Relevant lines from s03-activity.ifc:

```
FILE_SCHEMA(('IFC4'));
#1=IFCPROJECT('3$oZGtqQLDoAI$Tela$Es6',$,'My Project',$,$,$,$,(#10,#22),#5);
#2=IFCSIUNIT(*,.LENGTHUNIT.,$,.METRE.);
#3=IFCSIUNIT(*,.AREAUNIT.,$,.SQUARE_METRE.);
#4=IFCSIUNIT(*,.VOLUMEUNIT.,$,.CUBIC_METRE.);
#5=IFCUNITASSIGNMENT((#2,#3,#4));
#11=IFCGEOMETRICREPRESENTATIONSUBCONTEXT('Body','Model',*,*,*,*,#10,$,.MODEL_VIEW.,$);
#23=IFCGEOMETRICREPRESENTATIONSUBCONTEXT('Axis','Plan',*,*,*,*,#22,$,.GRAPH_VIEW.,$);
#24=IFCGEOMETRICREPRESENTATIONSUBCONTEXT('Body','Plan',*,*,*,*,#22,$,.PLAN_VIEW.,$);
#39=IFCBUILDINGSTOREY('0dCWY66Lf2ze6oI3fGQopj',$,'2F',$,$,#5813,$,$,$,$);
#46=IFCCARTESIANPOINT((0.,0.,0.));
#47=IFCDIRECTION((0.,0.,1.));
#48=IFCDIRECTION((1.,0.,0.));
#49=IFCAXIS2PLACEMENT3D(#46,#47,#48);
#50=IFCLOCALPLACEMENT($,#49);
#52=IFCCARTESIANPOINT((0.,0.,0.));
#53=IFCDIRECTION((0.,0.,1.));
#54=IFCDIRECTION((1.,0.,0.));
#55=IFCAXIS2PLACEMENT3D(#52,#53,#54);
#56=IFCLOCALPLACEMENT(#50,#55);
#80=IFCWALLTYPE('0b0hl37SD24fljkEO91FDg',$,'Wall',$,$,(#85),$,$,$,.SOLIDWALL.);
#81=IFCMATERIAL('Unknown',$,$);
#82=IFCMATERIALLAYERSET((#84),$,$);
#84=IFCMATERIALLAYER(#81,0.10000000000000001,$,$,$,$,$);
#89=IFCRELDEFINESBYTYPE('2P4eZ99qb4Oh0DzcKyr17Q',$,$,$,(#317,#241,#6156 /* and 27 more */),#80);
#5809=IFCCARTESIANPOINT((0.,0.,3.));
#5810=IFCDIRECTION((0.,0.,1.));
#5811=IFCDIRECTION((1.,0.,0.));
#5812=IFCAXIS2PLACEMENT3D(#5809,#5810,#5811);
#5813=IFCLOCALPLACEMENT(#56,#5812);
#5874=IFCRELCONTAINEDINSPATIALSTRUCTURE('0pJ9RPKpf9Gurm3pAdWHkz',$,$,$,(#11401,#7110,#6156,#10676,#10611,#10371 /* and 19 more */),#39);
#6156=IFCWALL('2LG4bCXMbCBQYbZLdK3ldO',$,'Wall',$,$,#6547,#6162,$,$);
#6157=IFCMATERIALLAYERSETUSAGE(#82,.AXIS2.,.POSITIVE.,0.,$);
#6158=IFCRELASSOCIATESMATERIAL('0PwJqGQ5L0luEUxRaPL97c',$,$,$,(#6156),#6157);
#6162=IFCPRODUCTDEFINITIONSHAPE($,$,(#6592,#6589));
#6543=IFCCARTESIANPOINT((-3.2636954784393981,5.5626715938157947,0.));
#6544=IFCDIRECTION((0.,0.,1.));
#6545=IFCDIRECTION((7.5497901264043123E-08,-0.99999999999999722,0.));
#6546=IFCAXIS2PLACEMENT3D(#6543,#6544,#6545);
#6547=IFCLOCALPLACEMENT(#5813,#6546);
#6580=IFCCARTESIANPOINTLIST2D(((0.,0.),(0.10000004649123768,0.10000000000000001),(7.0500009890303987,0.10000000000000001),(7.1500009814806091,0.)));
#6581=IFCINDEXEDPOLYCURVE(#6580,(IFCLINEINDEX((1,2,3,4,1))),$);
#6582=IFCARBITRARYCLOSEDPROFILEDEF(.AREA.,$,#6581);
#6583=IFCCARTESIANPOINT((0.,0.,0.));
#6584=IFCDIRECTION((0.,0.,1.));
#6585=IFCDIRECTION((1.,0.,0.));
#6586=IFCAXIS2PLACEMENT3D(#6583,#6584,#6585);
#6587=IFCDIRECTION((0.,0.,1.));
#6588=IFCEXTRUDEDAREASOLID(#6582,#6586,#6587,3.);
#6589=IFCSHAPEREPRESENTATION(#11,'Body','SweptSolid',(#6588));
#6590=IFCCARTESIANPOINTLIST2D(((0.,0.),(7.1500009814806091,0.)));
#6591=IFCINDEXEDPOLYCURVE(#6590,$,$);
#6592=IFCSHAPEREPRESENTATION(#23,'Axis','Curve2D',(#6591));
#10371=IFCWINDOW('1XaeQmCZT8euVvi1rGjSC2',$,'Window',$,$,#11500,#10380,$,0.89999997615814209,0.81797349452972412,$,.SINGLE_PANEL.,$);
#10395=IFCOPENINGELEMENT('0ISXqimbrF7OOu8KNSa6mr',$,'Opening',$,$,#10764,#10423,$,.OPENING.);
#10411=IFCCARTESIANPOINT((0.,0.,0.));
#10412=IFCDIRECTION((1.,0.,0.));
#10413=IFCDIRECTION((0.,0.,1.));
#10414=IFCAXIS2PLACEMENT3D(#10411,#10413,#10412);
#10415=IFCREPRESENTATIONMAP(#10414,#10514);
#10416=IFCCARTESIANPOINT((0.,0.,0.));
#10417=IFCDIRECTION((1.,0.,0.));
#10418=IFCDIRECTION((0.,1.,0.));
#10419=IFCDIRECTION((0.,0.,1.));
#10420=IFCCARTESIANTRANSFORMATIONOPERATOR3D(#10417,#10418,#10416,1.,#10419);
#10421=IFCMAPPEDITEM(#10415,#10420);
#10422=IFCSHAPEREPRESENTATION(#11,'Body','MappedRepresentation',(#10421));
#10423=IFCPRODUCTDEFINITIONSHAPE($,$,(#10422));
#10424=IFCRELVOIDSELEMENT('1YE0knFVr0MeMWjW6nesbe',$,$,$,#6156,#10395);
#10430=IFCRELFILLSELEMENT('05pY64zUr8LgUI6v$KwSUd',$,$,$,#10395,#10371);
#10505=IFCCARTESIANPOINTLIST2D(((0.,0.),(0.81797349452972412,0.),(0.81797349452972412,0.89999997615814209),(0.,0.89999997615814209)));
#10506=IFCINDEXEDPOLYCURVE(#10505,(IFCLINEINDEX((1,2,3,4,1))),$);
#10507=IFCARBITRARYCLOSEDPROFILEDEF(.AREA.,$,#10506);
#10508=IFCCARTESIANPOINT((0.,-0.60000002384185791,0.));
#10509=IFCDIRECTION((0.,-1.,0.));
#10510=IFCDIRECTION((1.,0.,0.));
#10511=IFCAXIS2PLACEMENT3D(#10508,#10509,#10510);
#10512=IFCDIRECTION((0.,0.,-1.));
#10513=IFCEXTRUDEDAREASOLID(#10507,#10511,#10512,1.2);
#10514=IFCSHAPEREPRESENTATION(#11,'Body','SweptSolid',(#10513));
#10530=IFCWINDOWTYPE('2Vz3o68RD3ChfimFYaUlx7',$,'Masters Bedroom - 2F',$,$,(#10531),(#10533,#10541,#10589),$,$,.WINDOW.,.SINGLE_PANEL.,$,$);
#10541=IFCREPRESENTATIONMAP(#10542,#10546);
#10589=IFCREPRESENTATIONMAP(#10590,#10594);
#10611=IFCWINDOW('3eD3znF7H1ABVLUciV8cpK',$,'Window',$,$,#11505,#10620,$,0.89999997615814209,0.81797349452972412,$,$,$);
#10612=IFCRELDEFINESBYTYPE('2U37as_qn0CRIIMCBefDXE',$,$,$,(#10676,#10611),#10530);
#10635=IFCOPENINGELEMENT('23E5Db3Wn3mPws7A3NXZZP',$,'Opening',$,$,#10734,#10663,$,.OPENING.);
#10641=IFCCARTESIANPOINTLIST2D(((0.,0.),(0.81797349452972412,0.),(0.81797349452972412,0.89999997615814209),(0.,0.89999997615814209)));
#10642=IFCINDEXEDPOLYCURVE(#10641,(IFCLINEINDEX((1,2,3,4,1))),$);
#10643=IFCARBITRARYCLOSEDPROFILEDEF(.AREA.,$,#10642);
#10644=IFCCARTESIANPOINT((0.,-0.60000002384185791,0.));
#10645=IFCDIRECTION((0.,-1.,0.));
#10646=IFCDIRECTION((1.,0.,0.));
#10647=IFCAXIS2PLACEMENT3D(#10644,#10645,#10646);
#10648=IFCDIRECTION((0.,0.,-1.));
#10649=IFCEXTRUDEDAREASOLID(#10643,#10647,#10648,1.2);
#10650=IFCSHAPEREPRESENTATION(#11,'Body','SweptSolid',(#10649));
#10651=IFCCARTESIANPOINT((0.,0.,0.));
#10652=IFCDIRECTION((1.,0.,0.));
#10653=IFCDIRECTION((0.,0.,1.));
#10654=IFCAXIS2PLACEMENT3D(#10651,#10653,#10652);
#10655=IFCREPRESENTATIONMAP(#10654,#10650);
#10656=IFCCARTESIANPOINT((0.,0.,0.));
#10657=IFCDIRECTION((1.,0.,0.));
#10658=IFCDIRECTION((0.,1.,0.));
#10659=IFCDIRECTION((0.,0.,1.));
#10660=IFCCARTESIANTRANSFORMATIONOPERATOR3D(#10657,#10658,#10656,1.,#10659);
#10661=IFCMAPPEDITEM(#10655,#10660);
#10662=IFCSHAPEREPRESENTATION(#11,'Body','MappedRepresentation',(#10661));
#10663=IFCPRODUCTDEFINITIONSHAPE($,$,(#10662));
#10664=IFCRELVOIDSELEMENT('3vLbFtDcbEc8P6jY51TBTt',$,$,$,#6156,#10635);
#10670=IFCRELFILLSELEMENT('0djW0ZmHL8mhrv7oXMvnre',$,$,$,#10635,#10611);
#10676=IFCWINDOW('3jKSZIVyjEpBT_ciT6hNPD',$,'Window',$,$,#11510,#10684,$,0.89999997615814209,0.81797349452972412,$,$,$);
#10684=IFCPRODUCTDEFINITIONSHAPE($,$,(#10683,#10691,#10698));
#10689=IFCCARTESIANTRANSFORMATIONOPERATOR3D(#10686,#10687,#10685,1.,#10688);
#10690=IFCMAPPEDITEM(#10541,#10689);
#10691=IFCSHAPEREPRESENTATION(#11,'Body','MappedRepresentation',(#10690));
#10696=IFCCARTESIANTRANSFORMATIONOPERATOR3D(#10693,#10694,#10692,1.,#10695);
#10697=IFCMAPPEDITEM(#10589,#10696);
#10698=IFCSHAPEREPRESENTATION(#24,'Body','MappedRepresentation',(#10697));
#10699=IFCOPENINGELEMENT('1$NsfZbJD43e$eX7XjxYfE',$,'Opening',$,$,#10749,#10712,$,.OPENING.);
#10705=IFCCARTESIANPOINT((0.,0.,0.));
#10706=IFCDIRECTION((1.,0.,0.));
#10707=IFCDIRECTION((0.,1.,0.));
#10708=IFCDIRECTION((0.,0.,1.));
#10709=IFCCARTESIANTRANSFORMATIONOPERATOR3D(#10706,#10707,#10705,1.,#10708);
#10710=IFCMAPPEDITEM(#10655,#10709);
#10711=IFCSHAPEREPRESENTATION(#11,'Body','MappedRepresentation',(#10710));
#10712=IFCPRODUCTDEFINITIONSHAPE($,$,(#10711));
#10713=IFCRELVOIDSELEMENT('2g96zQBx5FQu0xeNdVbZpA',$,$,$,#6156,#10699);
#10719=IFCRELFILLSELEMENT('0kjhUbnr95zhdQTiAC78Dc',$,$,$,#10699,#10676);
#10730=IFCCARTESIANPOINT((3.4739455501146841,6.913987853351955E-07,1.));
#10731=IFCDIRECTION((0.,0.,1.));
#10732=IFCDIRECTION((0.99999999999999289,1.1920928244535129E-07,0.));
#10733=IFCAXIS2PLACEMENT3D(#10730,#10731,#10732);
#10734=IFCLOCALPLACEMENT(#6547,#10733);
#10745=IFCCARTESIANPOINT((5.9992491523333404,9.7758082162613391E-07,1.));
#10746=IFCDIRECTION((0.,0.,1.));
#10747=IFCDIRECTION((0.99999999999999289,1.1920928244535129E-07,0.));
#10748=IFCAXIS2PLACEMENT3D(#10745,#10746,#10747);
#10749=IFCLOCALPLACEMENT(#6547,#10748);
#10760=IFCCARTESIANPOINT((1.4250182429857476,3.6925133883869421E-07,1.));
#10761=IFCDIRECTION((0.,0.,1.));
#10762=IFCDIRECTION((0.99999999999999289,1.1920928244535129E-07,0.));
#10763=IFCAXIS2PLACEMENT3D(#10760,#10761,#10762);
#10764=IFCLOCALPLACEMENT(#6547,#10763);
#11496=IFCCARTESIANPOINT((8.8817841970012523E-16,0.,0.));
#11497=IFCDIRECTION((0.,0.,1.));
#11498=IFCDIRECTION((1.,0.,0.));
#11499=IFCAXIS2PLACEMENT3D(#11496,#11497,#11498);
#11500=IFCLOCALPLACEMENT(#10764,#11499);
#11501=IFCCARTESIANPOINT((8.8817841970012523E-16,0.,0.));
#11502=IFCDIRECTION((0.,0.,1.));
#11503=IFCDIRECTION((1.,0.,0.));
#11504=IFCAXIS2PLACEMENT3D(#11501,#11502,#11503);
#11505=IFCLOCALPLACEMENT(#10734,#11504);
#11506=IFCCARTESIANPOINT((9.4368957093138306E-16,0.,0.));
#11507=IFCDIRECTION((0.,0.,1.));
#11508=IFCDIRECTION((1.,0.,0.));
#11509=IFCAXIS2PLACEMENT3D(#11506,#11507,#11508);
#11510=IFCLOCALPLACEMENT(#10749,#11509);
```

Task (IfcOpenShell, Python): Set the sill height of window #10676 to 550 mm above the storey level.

```python
import numpy as np
import ifcopenshell
import ifcopenshell.api.geometry
import ifcopenshell.geom
import ifcopenshell.util.element
import ifcopenshell.util.placement
import ifcopenshell.util.shape
import ifcopenshell.util.unit

model = ifcopenshell.open("s03-activity.ifc")
unit_scale = ifcopenshell.util.unit.calculate_unit_scale(model)

window = model.by_id(10676)
opening = window.FillsVoids[0].RelatingOpeningElement
storey = ifcopenshell.util.element.get_container(window, ifc_class="IfcBuildingStorey")
level = ifcopenshell.util.placement.get_local_placement(storey.ObjectPlacement)[2, 3]

# The opening's origin need not be at the sill, so measure its lowest point.
shape = ifcopenshell.geom.create_shape(ifcopenshell.geom.settings(), opening)
bottom = ifcopenshell.util.shape.get_shape_bottom_elevation(shape, shape.geometry) / unit_scale
dz = level + 0.55 / unit_scale - bottom

shift = np.array([0.0, 0.0, dz])
# The window is placed relative to its opening, so it follows when the opening moves.
matrix = ifcopenshell.util.placement.get_local_placement(opening.ObjectPlacement)
matrix[:3, 3] += shift
ifcopenshell.api.geometry.edit_object_placement(
    model, product=opening, matrix=matrix, is_si=False, should_transform_children=True
)

print(f"moved by {dz * unit_scale:+.3f} m")

model.write("s03-activity_v2.ifc")
```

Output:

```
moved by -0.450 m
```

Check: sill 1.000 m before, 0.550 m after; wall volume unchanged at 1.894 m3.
